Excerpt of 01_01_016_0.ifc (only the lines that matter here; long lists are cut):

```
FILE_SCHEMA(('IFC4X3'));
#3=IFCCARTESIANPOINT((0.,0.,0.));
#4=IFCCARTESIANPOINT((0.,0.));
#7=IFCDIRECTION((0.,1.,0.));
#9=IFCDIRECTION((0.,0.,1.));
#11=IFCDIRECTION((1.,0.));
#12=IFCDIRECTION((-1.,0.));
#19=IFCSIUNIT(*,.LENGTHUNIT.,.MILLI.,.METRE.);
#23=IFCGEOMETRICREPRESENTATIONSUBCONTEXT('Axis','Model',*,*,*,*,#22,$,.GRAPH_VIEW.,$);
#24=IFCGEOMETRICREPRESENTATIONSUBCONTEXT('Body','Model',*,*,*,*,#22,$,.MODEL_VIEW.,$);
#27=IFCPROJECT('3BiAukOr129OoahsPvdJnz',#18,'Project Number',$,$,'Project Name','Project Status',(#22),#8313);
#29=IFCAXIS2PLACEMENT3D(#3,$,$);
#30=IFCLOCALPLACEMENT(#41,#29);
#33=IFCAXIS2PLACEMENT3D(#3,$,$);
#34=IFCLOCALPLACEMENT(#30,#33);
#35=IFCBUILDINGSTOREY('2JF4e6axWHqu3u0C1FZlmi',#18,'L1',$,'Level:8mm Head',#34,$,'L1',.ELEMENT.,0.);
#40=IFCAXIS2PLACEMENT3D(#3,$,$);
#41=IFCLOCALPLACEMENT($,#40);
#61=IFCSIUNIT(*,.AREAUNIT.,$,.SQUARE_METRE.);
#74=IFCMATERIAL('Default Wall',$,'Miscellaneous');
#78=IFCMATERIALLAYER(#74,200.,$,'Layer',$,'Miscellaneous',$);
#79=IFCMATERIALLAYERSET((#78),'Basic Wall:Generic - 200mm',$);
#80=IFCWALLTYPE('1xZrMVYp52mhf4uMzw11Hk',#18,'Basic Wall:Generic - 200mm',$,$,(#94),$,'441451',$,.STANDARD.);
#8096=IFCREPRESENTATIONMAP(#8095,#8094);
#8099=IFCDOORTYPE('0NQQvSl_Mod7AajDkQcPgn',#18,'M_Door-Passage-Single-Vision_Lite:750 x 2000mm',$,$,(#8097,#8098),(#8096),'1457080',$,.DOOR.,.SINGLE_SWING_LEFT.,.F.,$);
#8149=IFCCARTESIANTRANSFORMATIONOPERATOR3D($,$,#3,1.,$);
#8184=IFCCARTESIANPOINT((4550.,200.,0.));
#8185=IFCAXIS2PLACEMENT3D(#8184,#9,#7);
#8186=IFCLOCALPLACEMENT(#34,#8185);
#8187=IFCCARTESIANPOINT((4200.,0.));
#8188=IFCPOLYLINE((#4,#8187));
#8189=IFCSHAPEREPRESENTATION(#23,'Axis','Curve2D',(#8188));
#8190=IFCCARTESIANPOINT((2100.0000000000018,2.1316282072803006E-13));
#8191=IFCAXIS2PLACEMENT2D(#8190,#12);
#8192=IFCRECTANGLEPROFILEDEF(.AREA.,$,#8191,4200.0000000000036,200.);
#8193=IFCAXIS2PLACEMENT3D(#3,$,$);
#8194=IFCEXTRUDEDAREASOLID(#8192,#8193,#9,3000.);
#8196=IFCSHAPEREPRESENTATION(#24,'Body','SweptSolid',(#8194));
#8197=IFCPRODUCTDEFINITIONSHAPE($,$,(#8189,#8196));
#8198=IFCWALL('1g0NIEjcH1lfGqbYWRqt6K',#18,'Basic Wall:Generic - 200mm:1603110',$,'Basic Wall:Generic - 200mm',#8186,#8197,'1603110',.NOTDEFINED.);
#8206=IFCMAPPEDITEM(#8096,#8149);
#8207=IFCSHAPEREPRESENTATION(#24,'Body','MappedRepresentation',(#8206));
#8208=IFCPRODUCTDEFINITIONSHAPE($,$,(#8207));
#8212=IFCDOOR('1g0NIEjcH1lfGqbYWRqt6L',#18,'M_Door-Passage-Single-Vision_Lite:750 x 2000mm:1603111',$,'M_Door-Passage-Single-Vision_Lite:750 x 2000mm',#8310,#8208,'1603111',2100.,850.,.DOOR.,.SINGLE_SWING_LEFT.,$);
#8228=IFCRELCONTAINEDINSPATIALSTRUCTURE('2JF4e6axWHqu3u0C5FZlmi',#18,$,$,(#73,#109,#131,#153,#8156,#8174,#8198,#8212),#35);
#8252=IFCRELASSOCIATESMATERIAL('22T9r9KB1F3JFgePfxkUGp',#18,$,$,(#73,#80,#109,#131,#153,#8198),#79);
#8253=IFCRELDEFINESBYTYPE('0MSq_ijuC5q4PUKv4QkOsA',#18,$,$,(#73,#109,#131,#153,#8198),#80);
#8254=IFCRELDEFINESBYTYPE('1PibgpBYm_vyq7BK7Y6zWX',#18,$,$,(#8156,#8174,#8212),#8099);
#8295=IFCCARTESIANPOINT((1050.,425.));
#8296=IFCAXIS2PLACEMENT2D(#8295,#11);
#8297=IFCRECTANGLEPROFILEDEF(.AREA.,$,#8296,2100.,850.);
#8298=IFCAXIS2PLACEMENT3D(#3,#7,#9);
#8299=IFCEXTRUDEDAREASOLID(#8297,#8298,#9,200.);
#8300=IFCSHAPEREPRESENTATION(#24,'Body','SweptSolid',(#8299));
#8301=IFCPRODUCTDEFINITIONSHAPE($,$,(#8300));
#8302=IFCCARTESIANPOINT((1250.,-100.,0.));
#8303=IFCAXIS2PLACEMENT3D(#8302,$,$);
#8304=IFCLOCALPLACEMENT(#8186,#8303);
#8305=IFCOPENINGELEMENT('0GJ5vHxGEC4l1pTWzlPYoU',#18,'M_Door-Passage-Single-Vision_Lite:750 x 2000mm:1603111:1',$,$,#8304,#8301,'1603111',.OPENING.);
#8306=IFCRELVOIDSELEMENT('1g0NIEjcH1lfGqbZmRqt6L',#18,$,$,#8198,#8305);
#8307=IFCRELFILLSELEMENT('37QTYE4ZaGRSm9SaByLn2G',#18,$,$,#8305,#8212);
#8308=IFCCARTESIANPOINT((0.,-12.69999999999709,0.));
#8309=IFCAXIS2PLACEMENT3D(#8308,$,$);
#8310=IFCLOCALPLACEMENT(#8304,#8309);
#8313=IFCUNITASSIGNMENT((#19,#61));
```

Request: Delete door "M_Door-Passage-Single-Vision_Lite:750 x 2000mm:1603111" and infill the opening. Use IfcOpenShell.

```python
import ifcopenshell
import ifcopenshell.api.feature
import ifcopenshell.api.root
import ifcopenshell.geom
import ifcopenshell.util.shape

model = ifcopenshell.open("01_01_016_0.ifc")
settings = ifcopenshell.geom.settings()


def volume(element):
    """Net volume in cubic metres, openings subtracted."""
    shape = ifcopenshell.geom.create_shape(settings, element)
    return ifcopenshell.util.shape.get_volume(shape.geometry)


door = model.by_guid("1g0NIEjcH1lfGqbYWRqt6L")
opening = door.FillsVoids[0].RelatingOpeningElement
wall = opening.VoidsElements[0].RelatingBuildingElement
before = volume(wall)

ifcopenshell.api.root.remove_product(model, product=door)
ifcopenshell.api.feature.remove_feature(model, feature=opening)

after = volume(wall)

print(f"wall volume {before:.3f} -> {after:.3f} m3")

model.write("01_01_016_0_rev.ifc")
```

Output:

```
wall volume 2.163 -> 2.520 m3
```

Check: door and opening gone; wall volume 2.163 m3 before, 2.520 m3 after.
